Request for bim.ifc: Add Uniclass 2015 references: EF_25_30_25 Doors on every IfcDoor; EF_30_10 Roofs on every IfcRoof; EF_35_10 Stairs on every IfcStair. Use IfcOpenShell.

First a look at what the model holds.

```python
import ifcopenshell

model = ifcopenshell.open("bim.ifc")
print(model.schema)
print("classifications:", [c.Name for c in model.by_type("IfcClassification")])
for ifc_class in ("IfcDoor", "IfcRoof", "IfcStair", "IfcWall", "IfcWindow"):
    print(ifc_class, len(model.by_type(ifc_class)))
```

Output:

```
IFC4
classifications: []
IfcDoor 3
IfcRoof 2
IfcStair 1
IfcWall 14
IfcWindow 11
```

```python
import ifcopenshell
import ifcopenshell.api.classification

model = ifcopenshell.open("bim.ifc")

system = ifcopenshell.api.classification.add_classification(model, classification="Uniclass 2015")

codes = {
    "IfcDoor": ("EF_25_30_25", "Doors"),
    "IfcRoof": ("EF_30_10", "Roofs"),
    "IfcStair": ("EF_35_10", "Stairs"),
}
for ifc_class, (code, name) in codes.items():
    products = model.by_type(ifc_class)
    ifcopenshell.api.classification.add_reference(
        model, products=products, classification=system, identification=code, name=name
    )
    print(code, len(products))

model.write("bim_v2.ifc")
```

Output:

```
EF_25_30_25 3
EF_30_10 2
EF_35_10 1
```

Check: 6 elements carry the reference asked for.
